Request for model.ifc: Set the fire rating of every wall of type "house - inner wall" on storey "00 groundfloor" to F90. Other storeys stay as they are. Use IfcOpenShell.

First a look at what the model holds.

```python
import ifcopenshell
import ifcopenshell.util.element

model = ifcopenshell.open("model.ifc")
print(model.schema)
storey = next(s for s in model.by_type("IfcBuildingStorey") if s.Name == "00 groundfloor")
walls = [e for e in ifcopenshell.util.element.get_decomposition(storey) if e.is_a("IfcWall")]
seen = {}
for e in walls:
    element_type = ifcopenshell.util.element.get_type(e)
    key = (element_type.Name if element_type != e and element_type else None, ifcopenshell.util.element.get_pset(e, "Pset_WallCommon", "FireRating"))
    seen[key] = seen.get(key, 0) + 1
for (name, value), count in sorted(seen.items(), key=str):
    print(count, "x", name, "|", value)
```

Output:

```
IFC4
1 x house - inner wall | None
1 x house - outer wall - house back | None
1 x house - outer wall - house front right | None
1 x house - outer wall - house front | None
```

```python
import ifcopenshell
import ifcopenshell.api.pset
import ifcopenshell.util.element

model = ifcopenshell.open("model.ifc")

storey = next(s for s in model.by_type("IfcBuildingStorey") if s.Name == "00 groundfloor")
walls = [e for e in ifcopenshell.util.element.get_decomposition(storey) if e.is_a("IfcWall")]

count = 0
for e in walls:
    element_type = ifcopenshell.util.element.get_type(e)
    if element_type in (None, e) or element_type.Name != "house - inner wall":
        continue
    # add_pset returns the element's existing set when there is one.
    pset = ifcopenshell.api.pset.add_pset(model, product=e, name="Pset_WallCommon")
    ifcopenshell.api.pset.edit_pset(model, pset=pset, properties={"FireRating": "F90"})
    count += 1

print(count, "walls updated")

model.write("model-out.ifc")
```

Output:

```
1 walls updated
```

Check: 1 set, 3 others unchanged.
